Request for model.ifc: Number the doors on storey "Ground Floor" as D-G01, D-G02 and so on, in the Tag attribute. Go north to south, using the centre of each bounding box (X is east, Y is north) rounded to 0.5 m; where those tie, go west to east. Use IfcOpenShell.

First a look at what the model holds.

```python
import ifcopenshell
import ifcopenshell.util.element
import ifcopenshell.util.placement

model = ifcopenshell.open("model.ifc")
print(model.schema)
storey = next(s for s in model.by_type("IfcBuildingStorey") if s.Name == "Ground Floor")
doors = [e for e in ifcopenshell.util.element.get_decomposition(storey) if e.is_a("IfcDoor")]
for e in sorted(doors, key=lambda e: e.id()):
    origin = ifcopenshell.util.placement.get_local_placement(e.ObjectPlacement)[:3, 3]
    print(e.id(), e.Tag, e.Name, origin.round(2) + 0.0, sep=" | ")
```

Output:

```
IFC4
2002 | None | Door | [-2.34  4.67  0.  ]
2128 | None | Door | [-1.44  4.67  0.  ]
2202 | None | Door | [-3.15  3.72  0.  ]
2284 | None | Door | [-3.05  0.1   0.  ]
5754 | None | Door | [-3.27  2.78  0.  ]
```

```python
import ifcopenshell
import ifcopenshell.geom
import ifcopenshell.util.element
import ifcopenshell.util.shape

model = ifcopenshell.open("model.ifc")
settings = ifcopenshell.geom.settings()
settings.set("use-world-coords", True)


def centre(element):
    shape = ifcopenshell.geom.create_shape(settings, element)
    return ifcopenshell.util.shape.get_bbox_centroid(shape.geometry)


storey = next(s for s in model.by_type("IfcBuildingStorey") if s.Name == "Ground Floor")
doors = [e for e in ifcopenshell.util.element.get_decomposition(storey) if e.is_a("IfcDoor")]

# Insertion points can sit at a corner or the storey origin, so sort by the geometry (in metres).
centres = {e: centre(e) for e in doors}
doors.sort(key=lambda e: (-round(centres[e][1] / 0.5), centres[e][0]))

for i, e in enumerate(doors, start=1):
    number = f"D-G{i:02d}"
    e.Tag = number
    print(e.id(), number)

model.write("model_updated.ifc")
```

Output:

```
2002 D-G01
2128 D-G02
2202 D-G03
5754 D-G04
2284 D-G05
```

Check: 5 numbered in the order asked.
